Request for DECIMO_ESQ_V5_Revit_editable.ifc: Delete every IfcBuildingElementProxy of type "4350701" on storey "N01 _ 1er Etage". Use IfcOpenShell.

First a look at what the model holds.

```python
import ifcopenshell
import ifcopenshell.util.element

model = ifcopenshell.open("DECIMO_ESQ_V5_Revit_editable.ifc")
print(model.schema)
storey = next(s for s in model.by_type("IfcBuildingStorey") if s.Name == "N01 _ 1er Etage")
proxies = [e for e in ifcopenshell.util.element.get_decomposition(storey) if e.is_a("IfcBuildingElementProxy")]
seen = {}
for e in proxies:
    element_type = ifcopenshell.util.element.get_type(e)
    name = element_type.Name if element_type not in (None, e) else None
    seen[name] = seen.get(name, 0) + 1
for name, count in sorted(seen.items(), key=str):
    print(count, "x", name)
```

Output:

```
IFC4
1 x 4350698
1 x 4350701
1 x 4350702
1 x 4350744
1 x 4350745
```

```python
import ifcopenshell
import ifcopenshell.api.root
import ifcopenshell.util.element

model = ifcopenshell.open("DECIMO_ESQ_V5_Revit_editable.ifc")

storey = next(s for s in model.by_type("IfcBuildingStorey") if s.Name == "N01 _ 1er Etage")
proxies = [e for e in ifcopenshell.util.element.get_decomposition(storey) if e.is_a("IfcBuildingElementProxy")]
targets = [e for e in proxies if (t := ifcopenshell.util.element.get_type(e)) not in (None, e) and t.Name == "4350701"]

for e in targets:
    ifcopenshell.api.root.remove_product(model, product=e)
print(len(targets), "removed")

model.write("DECIMO_ESQ_V5_Revit_editable-out.ifc")
```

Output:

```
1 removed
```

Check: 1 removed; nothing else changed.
